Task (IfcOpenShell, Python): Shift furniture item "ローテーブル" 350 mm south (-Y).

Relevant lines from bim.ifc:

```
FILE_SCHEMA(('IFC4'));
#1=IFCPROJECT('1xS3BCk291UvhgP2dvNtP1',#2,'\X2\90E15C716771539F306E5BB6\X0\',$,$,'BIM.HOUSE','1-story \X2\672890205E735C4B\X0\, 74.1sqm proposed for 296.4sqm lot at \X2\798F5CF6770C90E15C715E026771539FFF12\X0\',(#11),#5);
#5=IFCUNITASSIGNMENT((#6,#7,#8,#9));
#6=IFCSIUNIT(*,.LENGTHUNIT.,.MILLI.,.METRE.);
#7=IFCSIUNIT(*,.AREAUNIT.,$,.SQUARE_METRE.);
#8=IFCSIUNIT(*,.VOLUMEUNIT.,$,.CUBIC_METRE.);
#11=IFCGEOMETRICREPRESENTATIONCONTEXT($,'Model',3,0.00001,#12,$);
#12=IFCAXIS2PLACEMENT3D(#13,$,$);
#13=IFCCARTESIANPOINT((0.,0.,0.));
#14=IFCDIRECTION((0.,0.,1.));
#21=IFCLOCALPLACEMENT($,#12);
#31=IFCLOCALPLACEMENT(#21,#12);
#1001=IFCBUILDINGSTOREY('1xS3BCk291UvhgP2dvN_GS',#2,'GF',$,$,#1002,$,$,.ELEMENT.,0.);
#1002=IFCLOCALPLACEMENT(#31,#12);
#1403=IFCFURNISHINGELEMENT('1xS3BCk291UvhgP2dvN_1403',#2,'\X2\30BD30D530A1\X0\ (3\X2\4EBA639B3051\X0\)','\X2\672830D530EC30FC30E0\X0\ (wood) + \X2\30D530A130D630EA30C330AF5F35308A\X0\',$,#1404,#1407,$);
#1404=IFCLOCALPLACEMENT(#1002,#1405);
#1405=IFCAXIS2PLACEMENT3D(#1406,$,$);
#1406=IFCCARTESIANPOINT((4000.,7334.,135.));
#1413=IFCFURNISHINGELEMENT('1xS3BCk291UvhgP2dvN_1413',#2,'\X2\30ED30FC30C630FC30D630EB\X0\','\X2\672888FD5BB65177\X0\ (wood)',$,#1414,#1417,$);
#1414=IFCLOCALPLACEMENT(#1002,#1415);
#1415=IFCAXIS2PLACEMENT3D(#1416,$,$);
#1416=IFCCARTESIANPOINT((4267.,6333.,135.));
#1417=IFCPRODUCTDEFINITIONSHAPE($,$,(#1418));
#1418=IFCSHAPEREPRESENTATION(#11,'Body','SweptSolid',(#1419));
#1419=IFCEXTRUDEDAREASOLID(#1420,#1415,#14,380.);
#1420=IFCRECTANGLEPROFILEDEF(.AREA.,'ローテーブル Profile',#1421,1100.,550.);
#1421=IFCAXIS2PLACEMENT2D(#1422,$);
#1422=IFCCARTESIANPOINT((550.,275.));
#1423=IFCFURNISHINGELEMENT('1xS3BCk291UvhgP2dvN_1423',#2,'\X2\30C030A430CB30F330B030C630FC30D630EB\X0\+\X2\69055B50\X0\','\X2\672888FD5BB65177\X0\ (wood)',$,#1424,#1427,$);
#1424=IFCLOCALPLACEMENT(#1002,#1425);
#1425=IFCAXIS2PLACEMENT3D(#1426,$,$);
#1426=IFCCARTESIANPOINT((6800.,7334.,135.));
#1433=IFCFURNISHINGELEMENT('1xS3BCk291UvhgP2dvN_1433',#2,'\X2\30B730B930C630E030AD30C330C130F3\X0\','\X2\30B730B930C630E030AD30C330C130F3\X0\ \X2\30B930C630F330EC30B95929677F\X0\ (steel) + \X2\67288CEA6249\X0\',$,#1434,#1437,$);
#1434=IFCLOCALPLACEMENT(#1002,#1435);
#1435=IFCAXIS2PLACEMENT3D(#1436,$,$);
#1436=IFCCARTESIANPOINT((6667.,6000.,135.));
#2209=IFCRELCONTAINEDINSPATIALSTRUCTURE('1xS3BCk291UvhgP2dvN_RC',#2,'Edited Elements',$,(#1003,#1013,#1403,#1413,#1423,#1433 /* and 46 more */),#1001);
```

```python
import ifcopenshell
import ifcopenshell.api.geometry
import ifcopenshell.util.placement
import ifcopenshell.util.unit

model = ifcopenshell.open("bim.ifc")
unit_scale = ifcopenshell.util.unit.calculate_unit_scale(model)

item = model.by_guid("1xS3BCk291UvhgP2dvN_1413")
matrix = ifcopenshell.util.placement.get_local_placement(item.ObjectPlacement)
matrix[1, 3] -= 0.35 / unit_scale
ifcopenshell.api.geometry.edit_object_placement(model, product=item, matrix=matrix, is_si=False)

print(ifcopenshell.util.placement.get_local_placement(item.ObjectPlacement).round(3) + 0.0)

model.write("bim-out.ifc")
```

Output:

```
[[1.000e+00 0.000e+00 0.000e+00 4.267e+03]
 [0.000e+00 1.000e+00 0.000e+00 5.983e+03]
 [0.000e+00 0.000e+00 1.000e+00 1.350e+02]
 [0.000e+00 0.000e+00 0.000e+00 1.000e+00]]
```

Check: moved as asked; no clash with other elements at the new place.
